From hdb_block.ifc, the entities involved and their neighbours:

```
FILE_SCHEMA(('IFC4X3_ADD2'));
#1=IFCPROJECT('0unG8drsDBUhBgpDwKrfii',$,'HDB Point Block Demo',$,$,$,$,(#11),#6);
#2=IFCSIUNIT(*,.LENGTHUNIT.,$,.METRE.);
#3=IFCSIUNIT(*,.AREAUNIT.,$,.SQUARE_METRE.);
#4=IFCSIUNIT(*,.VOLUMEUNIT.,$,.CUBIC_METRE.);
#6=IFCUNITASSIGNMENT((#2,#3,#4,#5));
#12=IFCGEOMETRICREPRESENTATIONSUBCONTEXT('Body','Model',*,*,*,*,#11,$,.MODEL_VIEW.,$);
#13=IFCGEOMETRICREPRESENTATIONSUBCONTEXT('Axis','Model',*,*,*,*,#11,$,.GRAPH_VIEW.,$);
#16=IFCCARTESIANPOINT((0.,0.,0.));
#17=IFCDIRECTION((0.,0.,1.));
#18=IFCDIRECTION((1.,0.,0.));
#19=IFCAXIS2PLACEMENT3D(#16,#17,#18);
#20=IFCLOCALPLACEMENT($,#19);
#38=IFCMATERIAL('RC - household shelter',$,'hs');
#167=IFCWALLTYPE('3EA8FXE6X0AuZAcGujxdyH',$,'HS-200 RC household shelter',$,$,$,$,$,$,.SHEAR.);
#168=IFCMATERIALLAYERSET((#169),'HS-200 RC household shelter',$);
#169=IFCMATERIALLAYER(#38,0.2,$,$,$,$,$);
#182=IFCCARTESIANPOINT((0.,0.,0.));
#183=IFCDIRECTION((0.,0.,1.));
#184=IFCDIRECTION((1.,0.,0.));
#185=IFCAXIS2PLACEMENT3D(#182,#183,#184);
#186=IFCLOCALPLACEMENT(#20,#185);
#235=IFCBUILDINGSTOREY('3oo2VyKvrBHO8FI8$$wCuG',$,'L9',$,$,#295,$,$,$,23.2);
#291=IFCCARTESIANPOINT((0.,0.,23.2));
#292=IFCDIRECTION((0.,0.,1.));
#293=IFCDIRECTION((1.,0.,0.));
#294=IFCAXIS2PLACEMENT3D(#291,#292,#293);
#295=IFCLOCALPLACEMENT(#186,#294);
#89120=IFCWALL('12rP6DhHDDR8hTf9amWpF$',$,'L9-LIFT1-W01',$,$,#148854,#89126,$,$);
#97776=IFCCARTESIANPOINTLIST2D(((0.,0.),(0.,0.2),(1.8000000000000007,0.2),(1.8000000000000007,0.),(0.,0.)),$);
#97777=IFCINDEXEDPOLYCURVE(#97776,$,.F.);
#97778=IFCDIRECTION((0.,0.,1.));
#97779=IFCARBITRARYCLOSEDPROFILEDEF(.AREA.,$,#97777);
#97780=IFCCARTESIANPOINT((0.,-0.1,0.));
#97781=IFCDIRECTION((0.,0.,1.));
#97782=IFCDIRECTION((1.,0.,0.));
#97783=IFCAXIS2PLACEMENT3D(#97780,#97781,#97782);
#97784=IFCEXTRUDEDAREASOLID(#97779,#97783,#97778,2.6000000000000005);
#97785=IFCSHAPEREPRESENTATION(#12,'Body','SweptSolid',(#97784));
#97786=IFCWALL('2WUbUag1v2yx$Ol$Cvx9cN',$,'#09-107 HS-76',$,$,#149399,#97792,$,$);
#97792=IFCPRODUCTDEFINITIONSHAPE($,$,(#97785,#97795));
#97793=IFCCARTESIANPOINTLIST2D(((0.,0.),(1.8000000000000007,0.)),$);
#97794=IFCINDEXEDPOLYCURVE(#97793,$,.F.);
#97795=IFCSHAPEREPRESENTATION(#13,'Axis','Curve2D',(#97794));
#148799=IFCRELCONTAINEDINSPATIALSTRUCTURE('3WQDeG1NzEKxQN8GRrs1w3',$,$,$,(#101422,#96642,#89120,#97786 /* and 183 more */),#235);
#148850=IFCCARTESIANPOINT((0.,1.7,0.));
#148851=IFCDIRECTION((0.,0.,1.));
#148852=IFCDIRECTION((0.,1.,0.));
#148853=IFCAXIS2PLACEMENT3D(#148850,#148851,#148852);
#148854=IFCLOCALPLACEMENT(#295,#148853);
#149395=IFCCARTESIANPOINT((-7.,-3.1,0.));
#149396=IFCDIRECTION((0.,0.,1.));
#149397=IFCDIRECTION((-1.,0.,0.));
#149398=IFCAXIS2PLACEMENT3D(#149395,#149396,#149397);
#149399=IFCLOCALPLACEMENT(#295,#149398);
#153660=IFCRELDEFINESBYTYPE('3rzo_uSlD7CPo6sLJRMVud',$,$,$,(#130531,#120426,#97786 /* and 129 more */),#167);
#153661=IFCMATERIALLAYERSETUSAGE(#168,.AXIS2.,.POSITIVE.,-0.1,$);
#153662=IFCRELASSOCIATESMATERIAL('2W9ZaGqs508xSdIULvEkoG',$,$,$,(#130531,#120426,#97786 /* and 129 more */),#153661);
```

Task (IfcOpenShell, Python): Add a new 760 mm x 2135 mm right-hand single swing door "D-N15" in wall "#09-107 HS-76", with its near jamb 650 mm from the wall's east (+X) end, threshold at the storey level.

```python
import numpy as np
import ifcopenshell
import ifcopenshell.api.feature
import ifcopenshell.api.geometry
import ifcopenshell.api.root
import ifcopenshell.api.spatial
import ifcopenshell.geom
import ifcopenshell.util.element
import ifcopenshell.util.placement
import ifcopenshell.util.representation
import ifcopenshell.util.shape
import ifcopenshell.util.unit

model = ifcopenshell.open("hdb_block.ifc")
unit_scale = ifcopenshell.util.unit.calculate_unit_scale(model)
settings = ifcopenshell.geom.settings()


def volume(element):
    """Net volume in cubic metres, openings subtracted."""
    shape = ifcopenshell.geom.create_shape(settings, element)
    return ifcopenshell.util.shape.get_volume(shape.geometry)


wall = model.by_guid("2WUbUag1v2yx$Ol$Cvx9cN")
storey = ifcopenshell.util.element.get_container(wall, ifc_class="IfcBuildingStorey")
context = ifcopenshell.util.representation.get_context(model, "Model", "Body", "MODEL_VIEW")
before = volume(wall)

width, height, from_end, sill = 0.76, 2.135, 0.65, 0.0  # metres

# The wall runs along its own X axis, and the end named is its -X end.
wall_shape = ifcopenshell.geom.create_shape(settings, wall)
x, y, z = ifcopenshell.util.shape.get_vertices(wall_shape.geometry).T
start = x.min() + from_end
face, thickness = float(y.min()), float(y.max() - y.min())
wall_matrix = ifcopenshell.util.placement.get_local_placement(wall.ObjectPlacement)
level = ifcopenshell.util.placement.get_local_placement(storey.ObjectPlacement)[2, 3]


def in_wall(x, y):
    """Placement at x, y metres in the wall's axes, at sill height."""
    matrix = wall_matrix.copy()
    matrix[:, 3] = wall_matrix @ np.array([x / unit_scale, y / unit_scale, 0.0, 1.0])
    matrix[2, 3] = level + sill / unit_scale
    return matrix


# Opening: a box that overshoots both wall faces by 50 mm.
opening = ifcopenshell.api.root.create_entity(model, ifc_class="IfcOpeningElement", predefined_type="OPENING")
box = ifcopenshell.api.geometry.add_wall_representation(
    model, context=context, length=width, height=height, thickness=thickness + 0.1
)
ifcopenshell.api.geometry.assign_representation(model, product=opening, representation=box)
ifcopenshell.api.geometry.edit_object_placement(model, product=opening, matrix=in_wall(start, face - 0.05), is_si=False)
ifcopenshell.api.feature.add_feature(model, feature=opening, element=wall)

door = ifcopenshell.api.root.create_entity(model, ifc_class="IfcDoor", name="D-N15", predefined_type="DOOR")
door.OverallWidth, door.OverallHeight = width / unit_scale, height / unit_scale
door.OperationType = "SINGLE_SWING_RIGHT"
body = ifcopenshell.api.geometry.add_door_representation(
    model,
    context=context,
    overall_width=door.OverallWidth,
    overall_height=door.OverallHeight,
    operation_type="SINGLE_SWING_RIGHT",
    lining_properties={"LiningDepth": thickness / unit_scale, "ThresholdDepth": thickness / unit_scale},
)
ifcopenshell.api.geometry.assign_representation(model, product=door, representation=body)
ifcopenshell.api.spatial.assign_container(model, products=[door], relating_structure=storey)
ifcopenshell.api.feature.add_filling(model, opening=opening, element=door)

# The lining spans the wall, so the door starts at the wall face.
ifcopenshell.api.geometry.edit_object_placement(model, product=door, matrix=in_wall(start, face), is_si=False)

after = volume(wall)

print(f"wall volume {before:.3f} -> {after:.3f} m3")

model.write("hdb_block_updated.ifc")
```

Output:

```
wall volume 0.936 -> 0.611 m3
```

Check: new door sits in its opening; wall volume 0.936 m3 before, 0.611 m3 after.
